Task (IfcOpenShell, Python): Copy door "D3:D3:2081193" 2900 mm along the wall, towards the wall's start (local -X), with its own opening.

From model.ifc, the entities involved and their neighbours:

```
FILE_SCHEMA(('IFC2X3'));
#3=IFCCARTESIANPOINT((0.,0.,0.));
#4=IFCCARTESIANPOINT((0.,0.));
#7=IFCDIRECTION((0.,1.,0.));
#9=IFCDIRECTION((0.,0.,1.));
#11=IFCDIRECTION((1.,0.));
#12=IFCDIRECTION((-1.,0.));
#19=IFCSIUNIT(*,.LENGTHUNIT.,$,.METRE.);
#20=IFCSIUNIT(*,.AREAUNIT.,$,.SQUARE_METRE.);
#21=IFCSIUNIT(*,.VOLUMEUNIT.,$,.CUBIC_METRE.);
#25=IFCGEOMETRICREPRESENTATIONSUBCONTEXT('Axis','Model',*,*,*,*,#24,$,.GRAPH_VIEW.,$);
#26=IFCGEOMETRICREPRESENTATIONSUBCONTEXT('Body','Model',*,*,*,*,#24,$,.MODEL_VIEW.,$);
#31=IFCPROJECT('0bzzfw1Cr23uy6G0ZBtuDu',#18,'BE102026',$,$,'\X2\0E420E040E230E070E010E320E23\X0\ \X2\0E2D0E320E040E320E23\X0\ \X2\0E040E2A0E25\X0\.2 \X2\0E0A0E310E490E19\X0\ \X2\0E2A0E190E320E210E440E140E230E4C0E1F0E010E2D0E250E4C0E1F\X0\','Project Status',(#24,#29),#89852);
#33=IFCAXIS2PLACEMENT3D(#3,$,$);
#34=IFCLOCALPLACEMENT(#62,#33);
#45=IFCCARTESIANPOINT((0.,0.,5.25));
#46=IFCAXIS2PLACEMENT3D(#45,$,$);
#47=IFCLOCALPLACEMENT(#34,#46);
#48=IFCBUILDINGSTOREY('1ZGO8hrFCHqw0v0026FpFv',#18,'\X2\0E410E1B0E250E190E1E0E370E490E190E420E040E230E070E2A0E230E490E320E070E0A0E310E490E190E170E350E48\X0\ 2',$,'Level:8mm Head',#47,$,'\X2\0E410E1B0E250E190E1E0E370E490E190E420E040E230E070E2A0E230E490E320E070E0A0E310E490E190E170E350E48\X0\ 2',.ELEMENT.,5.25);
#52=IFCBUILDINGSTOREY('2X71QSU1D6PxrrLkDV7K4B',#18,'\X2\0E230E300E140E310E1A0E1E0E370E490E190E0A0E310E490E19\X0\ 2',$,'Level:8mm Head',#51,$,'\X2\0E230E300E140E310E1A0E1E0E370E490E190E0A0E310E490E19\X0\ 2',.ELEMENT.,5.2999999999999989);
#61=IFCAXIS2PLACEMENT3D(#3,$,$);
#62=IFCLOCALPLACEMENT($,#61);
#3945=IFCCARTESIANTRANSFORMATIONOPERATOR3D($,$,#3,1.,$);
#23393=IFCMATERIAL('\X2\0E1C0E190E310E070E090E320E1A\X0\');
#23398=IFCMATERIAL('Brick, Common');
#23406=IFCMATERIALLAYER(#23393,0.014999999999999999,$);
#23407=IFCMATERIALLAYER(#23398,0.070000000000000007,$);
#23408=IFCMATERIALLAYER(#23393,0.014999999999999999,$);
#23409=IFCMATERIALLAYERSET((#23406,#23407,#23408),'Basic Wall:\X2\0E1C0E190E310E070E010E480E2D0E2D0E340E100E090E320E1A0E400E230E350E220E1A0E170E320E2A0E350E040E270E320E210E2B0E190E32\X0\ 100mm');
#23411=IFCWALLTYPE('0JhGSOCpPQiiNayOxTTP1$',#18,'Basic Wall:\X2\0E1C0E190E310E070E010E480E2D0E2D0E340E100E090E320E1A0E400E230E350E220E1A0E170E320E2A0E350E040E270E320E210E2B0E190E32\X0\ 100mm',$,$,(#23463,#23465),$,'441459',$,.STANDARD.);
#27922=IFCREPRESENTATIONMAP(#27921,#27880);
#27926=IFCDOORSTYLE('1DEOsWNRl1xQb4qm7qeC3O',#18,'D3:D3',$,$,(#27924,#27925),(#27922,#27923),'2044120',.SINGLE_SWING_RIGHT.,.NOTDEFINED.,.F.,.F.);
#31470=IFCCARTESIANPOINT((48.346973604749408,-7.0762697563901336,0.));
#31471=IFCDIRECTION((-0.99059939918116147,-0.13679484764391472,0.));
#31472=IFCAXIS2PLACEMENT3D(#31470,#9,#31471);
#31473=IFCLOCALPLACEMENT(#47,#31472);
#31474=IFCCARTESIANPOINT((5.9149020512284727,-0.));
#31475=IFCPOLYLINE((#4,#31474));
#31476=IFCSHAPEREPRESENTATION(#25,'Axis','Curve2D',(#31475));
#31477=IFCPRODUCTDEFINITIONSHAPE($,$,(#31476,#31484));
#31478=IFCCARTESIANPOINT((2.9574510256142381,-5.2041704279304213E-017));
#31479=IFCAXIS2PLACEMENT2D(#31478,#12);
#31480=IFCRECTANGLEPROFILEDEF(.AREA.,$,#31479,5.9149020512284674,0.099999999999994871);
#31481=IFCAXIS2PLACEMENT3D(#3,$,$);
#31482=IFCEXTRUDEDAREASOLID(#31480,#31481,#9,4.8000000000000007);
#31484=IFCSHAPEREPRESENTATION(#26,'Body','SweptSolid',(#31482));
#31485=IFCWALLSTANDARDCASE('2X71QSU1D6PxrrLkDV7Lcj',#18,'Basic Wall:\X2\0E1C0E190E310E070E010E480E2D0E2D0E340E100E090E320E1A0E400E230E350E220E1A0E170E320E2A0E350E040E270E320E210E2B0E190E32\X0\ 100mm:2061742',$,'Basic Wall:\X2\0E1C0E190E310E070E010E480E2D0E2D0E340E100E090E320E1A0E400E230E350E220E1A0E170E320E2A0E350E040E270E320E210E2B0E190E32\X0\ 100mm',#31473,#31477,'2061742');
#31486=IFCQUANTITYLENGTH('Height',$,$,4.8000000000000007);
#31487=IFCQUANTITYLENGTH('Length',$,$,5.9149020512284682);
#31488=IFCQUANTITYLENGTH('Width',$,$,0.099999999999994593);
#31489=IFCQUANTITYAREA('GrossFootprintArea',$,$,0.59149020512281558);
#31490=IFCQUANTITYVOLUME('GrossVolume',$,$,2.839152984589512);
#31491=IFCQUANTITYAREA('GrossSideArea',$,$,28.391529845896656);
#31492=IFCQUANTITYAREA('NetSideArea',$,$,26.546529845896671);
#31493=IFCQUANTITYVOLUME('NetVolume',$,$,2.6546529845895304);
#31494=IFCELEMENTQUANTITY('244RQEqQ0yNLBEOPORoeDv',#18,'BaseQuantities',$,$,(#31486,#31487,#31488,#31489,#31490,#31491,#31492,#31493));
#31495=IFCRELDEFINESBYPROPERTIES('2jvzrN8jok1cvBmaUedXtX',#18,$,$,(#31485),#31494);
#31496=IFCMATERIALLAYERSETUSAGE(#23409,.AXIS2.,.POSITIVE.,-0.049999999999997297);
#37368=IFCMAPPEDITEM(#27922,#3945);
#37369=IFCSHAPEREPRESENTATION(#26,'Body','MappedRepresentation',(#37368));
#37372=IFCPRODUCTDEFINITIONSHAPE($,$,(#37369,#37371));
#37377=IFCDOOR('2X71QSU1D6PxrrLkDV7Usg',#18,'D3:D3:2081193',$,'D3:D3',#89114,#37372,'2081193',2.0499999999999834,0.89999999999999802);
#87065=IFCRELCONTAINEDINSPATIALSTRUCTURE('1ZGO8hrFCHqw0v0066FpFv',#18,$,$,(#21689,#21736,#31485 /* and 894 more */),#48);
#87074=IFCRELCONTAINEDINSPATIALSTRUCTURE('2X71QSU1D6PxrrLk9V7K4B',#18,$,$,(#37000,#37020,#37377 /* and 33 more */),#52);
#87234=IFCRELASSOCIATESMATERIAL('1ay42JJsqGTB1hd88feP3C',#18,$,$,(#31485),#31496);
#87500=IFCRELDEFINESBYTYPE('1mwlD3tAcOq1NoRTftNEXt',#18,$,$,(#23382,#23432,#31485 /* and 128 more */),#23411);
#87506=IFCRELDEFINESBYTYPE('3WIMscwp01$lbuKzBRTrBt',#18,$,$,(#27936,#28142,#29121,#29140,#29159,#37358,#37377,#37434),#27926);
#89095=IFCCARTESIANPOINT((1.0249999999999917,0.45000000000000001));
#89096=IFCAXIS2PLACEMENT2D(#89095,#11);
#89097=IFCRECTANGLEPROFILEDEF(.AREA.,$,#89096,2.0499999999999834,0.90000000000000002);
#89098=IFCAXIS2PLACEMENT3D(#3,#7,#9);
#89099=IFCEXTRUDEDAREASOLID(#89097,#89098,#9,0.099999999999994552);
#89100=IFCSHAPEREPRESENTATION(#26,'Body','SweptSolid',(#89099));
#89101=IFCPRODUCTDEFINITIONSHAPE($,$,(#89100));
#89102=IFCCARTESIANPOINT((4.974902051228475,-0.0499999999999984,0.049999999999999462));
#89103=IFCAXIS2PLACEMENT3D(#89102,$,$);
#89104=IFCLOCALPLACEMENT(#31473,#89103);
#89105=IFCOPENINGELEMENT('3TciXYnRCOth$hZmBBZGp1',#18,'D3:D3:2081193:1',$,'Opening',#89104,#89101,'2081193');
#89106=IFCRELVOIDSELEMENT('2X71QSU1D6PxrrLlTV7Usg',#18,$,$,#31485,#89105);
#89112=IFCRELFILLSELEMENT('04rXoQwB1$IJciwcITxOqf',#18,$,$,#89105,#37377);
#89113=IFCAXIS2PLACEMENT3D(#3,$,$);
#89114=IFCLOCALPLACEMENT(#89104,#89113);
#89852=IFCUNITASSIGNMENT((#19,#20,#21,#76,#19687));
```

```python
import ifcopenshell
import ifcopenshell.api.feature
import ifcopenshell.api.geometry
import ifcopenshell.api.pset
import ifcopenshell.api.root
import ifcopenshell.geom
import ifcopenshell.util.element
import ifcopenshell.util.placement
import ifcopenshell.util.shape
import ifcopenshell.util.unit

model = ifcopenshell.open("model.ifc")
unit_scale = ifcopenshell.util.unit.calculate_unit_scale(model)
area_scale = ifcopenshell.util.unit.calculate_unit_scale(model, "AREAUNIT")
volume_scale = ifcopenshell.util.unit.calculate_unit_scale(model, "VOLUMEUNIT")
settings = ifcopenshell.geom.settings()


def volume(element):
    """Net volume in cubic metres, openings subtracted."""
    shape = ifcopenshell.geom.create_shape(settings, element)
    return ifcopenshell.util.shape.get_volume(shape.geometry)


def reuse_history(source, copy):
    """copy_class also copies each property set's owner history, people and application; keep the originals."""
    for rel in copy.IsDefinedBy:
        if rel.is_a("IfcRelDefinesByProperties") and (history := rel.RelatingPropertyDefinition.OwnerHistory):
            rel.RelatingPropertyDefinition.OwnerHistory = source.OwnerHistory
            ifcopenshell.util.element.remove_deep2(model, history)


door = model.by_guid("2X71QSU1D6PxrrLkDV7Usg")
opening = door.FillsVoids[0].RelatingOpeningElement
wall = opening.VoidsElements[0].RelatingBuildingElement
before = volume(wall)
shift = ifcopenshell.util.placement.get_local_placement(wall.ObjectPlacement)[:3, 0] * -2.9 / unit_scale

# copy_class copies the void relationship, type, container and properties, but no geometry.
new_opening = ifcopenshell.api.root.copy_class(model, product=opening)
new_opening.Representation = ifcopenshell.util.element.copy_deep(
    model, opening.Representation, exclude=["IfcGeometricRepresentationContext", "IfcRepresentationMap"]
)
new_opening.Name = "D3:D3"
new_opening.Tag = None
reuse_history(opening, new_opening)
new_door = ifcopenshell.api.root.copy_class(model, product=door)
new_door.Representation = ifcopenshell.util.element.copy_deep(
    model, door.Representation, exclude=["IfcGeometricRepresentationContext", "IfcRepresentationMap"]
)
new_door.Name = "D3:D3"
new_door.Tag = None
reuse_history(door, new_door)
fills = ifcopenshell.api.feature.add_filling(model, opening=new_opening, element=new_door)
fills.OwnerHistory = new_door.OwnerHistory  # required in IFC2X3

for old, new in ((opening, new_opening), (door, new_door)):
    matrix = ifcopenshell.util.placement.get_local_placement(old.ObjectPlacement)
    matrix[:3, 3] += shift
    ifcopenshell.api.geometry.edit_object_placement(model, product=new, matrix=matrix, is_si=False)

after = volume(wall)
thickness = 0.1  # wall thickness in metres

# Update the wall's stored quantities.
qto = model.by_id(ifcopenshell.util.element.get_pset(wall, "BaseQuantities", should_inherit=False)["id"])
ifcopenshell.api.pset.edit_qto(model, qto=qto, properties={
    "NetSideArea": after / thickness / area_scale,
    "NetVolume": after / volume_scale,
})

print(f"wall volume {before:.3f} -> {after:.3f} m3")

model.write("model_updated.ifc")
```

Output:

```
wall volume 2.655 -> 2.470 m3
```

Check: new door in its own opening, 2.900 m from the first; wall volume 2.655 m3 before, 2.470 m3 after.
